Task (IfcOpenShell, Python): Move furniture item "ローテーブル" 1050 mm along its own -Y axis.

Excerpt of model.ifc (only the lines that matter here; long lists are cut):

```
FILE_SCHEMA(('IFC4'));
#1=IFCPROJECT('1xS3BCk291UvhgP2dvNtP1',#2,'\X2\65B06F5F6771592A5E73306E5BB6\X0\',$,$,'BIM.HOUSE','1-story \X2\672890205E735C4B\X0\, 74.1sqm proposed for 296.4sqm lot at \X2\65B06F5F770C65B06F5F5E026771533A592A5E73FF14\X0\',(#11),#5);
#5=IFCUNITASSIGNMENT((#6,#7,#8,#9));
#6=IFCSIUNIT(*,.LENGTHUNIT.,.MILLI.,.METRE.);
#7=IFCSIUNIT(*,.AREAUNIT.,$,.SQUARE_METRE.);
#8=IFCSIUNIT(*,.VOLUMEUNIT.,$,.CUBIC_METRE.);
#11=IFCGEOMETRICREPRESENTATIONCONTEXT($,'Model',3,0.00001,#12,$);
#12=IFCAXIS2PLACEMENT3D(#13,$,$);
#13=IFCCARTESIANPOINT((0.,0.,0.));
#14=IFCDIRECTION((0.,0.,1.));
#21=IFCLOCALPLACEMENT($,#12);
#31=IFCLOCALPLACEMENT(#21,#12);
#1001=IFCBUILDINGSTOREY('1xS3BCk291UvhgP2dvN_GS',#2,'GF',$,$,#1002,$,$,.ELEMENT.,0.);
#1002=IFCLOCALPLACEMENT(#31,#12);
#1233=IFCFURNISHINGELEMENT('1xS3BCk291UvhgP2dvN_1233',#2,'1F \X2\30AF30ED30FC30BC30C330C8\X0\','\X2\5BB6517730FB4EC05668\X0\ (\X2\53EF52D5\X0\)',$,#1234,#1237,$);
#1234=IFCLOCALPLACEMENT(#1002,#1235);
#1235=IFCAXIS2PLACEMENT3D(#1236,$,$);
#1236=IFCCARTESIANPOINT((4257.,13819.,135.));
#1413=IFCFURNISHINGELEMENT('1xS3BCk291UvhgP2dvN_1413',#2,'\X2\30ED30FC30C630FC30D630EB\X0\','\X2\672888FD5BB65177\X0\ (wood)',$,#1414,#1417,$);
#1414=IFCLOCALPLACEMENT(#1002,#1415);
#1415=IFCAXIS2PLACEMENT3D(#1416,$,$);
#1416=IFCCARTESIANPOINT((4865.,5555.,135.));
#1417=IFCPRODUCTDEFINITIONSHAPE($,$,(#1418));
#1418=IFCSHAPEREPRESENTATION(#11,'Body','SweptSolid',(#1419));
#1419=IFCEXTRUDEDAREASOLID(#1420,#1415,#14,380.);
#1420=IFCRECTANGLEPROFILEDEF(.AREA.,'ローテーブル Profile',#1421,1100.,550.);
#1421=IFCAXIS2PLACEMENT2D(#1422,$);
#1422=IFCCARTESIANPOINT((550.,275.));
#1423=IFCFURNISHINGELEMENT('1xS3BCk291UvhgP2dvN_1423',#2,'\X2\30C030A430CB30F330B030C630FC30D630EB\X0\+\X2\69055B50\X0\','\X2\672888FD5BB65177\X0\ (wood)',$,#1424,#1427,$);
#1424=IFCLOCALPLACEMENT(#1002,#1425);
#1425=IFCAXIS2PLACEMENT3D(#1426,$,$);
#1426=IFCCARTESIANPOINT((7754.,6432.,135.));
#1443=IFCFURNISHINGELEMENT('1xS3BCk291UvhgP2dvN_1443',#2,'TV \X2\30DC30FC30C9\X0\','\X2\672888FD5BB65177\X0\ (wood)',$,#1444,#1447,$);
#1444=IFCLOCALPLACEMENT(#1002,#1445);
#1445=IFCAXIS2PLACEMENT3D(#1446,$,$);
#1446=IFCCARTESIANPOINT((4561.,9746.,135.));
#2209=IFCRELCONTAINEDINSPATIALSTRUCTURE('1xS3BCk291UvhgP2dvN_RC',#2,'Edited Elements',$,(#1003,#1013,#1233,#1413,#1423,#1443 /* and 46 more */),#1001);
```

```python
import ifcopenshell
import ifcopenshell.api.geometry
import ifcopenshell.util.placement

model = ifcopenshell.open("model.ifc")

item = model.by_id(1413)
matrix = ifcopenshell.util.placement.get_local_placement(item.ObjectPlacement)
matrix[:3, 3] -= matrix[:3, 1] * 1050.0
ifcopenshell.api.geometry.edit_object_placement(model, product=item, matrix=matrix, is_si=False)

print(ifcopenshell.util.placement.get_local_placement(item.ObjectPlacement).round(3) + 0.0)

model.write("model_updated.ifc")
```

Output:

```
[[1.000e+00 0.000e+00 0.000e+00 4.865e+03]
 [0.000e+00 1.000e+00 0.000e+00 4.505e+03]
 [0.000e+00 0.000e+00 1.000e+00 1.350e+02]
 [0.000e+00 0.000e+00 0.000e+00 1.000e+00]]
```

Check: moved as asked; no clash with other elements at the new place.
